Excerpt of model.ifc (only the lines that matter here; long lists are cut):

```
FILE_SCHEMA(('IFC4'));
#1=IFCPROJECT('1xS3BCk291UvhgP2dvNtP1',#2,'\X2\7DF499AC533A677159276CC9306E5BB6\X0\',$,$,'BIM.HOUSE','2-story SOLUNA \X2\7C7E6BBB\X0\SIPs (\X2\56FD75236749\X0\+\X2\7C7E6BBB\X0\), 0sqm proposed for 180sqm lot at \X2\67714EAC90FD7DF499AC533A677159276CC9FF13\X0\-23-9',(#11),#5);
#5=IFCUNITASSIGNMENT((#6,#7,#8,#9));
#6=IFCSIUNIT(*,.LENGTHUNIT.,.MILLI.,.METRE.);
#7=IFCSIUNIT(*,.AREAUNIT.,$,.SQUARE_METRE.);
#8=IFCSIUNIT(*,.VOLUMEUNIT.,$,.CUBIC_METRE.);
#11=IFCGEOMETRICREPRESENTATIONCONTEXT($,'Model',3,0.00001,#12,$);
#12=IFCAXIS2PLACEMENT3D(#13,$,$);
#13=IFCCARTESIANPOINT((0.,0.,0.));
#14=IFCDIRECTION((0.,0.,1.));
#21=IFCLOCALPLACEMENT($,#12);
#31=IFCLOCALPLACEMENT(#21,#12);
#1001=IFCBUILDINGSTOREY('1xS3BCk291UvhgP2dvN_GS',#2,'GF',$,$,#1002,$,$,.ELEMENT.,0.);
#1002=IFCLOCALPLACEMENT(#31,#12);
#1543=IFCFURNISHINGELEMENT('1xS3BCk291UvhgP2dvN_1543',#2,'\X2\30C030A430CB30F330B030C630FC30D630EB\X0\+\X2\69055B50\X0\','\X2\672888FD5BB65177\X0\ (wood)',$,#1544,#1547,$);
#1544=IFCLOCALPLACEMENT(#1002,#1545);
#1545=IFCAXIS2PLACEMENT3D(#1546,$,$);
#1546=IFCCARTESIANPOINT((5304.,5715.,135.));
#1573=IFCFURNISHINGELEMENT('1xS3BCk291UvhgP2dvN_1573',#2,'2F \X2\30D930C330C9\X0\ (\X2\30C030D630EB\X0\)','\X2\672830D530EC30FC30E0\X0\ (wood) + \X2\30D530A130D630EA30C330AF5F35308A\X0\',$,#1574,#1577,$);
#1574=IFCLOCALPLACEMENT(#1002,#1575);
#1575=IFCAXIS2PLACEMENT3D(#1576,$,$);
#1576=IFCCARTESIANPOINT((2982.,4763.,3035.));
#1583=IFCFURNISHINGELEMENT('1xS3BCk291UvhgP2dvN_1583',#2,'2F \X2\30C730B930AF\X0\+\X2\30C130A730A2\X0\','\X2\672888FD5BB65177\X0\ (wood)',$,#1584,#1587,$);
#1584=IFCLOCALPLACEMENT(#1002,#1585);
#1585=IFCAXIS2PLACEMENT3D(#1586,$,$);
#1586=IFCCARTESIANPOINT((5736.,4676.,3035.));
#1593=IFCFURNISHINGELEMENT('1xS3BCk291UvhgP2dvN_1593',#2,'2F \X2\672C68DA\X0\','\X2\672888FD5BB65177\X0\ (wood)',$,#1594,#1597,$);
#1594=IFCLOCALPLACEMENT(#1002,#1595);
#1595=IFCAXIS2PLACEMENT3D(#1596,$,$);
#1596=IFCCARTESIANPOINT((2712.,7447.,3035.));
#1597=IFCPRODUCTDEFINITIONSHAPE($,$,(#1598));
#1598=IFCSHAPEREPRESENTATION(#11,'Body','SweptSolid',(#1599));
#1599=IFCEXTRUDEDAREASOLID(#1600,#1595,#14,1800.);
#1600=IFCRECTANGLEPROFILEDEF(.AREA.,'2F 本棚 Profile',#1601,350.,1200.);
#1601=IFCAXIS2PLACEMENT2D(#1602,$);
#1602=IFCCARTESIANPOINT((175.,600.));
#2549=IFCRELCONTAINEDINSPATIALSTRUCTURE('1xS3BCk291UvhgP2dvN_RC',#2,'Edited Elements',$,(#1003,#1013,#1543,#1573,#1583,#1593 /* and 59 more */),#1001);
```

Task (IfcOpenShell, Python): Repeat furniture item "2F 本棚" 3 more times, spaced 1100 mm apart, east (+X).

```python
import numpy as np
import ifcopenshell
import ifcopenshell.api.geometry
import ifcopenshell.api.root
import ifcopenshell.util.element
import ifcopenshell.util.placement

model = ifcopenshell.open("model.ifc")


def reuse_history(source, copy):
    """copy_class also copies each property set's owner history, people and application; keep the originals."""
    for rel in copy.IsDefinedBy:
        if rel.is_a("IfcRelDefinesByProperties") and (history := rel.RelatingPropertyDefinition.OwnerHistory):
            rel.RelatingPropertyDefinition.OwnerHistory = source.OwnerHistory
            ifcopenshell.util.element.remove_deep2(model, history)


source = model.by_id(1593)
base = ifcopenshell.util.placement.get_local_placement(source.ObjectPlacement)
step = np.array([1.0, 0.0, 0.0]) * 1100.0

for i in range(1, 4):
    copy = ifcopenshell.api.root.copy_class(model, product=source)
    copy.Representation = ifcopenshell.util.element.copy_deep(
        model, source.Representation, exclude=["IfcGeometricRepresentationContext", "IfcRepresentationMap"]
    )
    reuse_history(source, copy)
    matrix = base.copy()
    matrix[:3, 3] += i * step
    print("added at", matrix[:3, 3].round(3) + 0.0)
    ifcopenshell.api.geometry.edit_object_placement(model, product=copy, matrix=matrix, is_si=False)

model.write("model_v2.ifc")
```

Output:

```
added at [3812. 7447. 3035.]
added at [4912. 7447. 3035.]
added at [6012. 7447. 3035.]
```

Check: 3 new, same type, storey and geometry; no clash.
